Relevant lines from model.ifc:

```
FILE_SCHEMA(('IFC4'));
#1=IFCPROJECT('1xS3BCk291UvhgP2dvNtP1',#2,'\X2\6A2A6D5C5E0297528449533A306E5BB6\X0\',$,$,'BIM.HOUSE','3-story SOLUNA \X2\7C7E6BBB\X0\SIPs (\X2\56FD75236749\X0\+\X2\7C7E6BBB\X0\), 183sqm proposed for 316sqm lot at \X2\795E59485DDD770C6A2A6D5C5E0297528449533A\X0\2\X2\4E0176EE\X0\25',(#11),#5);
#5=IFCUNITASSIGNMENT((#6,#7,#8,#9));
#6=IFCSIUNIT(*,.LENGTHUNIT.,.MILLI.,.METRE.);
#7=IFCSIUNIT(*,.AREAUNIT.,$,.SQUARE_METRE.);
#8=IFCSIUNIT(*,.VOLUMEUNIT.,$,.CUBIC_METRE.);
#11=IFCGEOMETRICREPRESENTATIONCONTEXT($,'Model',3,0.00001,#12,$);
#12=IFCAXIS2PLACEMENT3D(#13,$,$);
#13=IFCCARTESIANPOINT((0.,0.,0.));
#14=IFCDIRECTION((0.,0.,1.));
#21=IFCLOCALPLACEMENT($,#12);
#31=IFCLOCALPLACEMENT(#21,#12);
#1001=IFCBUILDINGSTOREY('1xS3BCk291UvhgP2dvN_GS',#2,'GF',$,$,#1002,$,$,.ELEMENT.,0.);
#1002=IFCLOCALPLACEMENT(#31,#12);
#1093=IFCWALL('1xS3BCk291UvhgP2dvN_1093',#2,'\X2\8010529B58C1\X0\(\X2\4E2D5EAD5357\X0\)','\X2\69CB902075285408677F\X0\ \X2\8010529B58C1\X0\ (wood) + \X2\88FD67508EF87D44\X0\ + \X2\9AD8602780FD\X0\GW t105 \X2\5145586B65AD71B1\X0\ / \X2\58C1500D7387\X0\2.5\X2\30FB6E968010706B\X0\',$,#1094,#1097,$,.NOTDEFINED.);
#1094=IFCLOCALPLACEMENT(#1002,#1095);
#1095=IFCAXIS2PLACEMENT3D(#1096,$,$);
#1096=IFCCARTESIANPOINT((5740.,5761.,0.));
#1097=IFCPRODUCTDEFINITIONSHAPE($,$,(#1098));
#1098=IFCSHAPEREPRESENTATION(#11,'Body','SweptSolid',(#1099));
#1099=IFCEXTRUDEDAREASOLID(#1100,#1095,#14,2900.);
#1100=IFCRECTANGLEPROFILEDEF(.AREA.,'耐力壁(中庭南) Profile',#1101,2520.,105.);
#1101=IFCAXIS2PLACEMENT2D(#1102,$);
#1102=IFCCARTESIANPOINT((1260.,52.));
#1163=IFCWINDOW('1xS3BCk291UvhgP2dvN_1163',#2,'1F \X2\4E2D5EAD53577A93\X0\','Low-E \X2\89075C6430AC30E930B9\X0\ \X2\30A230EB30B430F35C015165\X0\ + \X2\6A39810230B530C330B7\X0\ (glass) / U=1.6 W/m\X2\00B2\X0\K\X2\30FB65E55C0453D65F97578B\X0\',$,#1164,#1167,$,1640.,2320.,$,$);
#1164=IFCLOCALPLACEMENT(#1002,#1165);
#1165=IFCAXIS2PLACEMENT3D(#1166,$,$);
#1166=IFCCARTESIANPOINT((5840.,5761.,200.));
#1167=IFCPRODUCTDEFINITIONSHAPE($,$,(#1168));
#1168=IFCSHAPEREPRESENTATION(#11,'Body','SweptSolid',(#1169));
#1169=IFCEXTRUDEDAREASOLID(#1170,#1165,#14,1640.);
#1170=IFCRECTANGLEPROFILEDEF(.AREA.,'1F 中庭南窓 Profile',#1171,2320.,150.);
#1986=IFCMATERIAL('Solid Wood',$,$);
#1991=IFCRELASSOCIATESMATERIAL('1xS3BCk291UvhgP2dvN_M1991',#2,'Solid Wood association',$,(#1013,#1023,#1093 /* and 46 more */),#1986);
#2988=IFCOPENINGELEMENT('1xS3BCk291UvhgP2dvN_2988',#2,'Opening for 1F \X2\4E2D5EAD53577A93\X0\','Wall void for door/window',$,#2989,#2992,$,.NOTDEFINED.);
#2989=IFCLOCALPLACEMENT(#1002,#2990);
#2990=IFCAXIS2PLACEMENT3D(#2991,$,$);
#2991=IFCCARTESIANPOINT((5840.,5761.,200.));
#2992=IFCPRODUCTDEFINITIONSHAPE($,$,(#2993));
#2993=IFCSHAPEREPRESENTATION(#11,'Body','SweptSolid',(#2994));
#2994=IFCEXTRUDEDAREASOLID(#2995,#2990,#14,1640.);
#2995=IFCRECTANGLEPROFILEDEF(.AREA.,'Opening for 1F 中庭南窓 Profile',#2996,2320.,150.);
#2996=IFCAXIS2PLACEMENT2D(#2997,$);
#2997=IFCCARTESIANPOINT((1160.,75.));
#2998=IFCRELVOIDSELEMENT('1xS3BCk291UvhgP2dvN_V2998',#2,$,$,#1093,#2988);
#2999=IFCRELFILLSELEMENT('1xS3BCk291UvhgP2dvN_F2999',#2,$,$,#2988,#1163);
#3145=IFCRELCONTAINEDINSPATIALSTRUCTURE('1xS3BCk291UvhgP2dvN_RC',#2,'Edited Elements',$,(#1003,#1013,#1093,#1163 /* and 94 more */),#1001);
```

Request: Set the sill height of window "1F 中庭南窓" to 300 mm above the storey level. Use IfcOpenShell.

```python
import numpy as np
import ifcopenshell
import ifcopenshell.api.geometry
import ifcopenshell.geom
import ifcopenshell.util.element
import ifcopenshell.util.placement
import ifcopenshell.util.shape
import ifcopenshell.util.unit

model = ifcopenshell.open("model.ifc")
unit_scale = ifcopenshell.util.unit.calculate_unit_scale(model)

window = model.by_guid("1xS3BCk291UvhgP2dvN_1163")
opening = window.FillsVoids[0].RelatingOpeningElement
storey = ifcopenshell.util.element.get_container(window, ifc_class="IfcBuildingStorey")
level = ifcopenshell.util.placement.get_local_placement(storey.ObjectPlacement)[2, 3]

# The opening's origin need not be at the sill, so measure its lowest point.
shape = ifcopenshell.geom.create_shape(ifcopenshell.geom.settings(), opening)
bottom = ifcopenshell.util.shape.get_shape_bottom_elevation(shape, shape.geometry) / unit_scale
dz = level + 0.3 / unit_scale - bottom

shift = np.array([0.0, 0.0, dz])
# The window is not placed relative to its opening, so move both.
for product in (opening, window):
    matrix = ifcopenshell.util.placement.get_local_placement(product.ObjectPlacement)
    matrix[:3, 3] += shift
    ifcopenshell.api.geometry.edit_object_placement(model, product=product, matrix=matrix, is_si=False)

print(f"moved by {dz * unit_scale:+.3f} m")

model.write("model_edited.ifc")
```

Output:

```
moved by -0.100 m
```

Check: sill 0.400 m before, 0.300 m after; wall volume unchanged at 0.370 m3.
